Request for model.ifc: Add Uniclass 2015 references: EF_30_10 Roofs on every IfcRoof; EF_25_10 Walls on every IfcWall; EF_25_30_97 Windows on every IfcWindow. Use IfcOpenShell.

First a look at what the model holds.

```python
import ifcopenshell

model = ifcopenshell.open("model.ifc")
print(model.schema)
print("classifications:", [c.Name for c in model.by_type("IfcClassification")])
for ifc_class in ("IfcDoor", "IfcRoof", "IfcStair", "IfcWall", "IfcWindow"):
    print(ifc_class, len(model.by_type(ifc_class)))
```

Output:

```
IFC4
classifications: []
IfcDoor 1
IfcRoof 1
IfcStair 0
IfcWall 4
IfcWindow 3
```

```python
import ifcopenshell
import ifcopenshell.api.classification

model = ifcopenshell.open("model.ifc")

system = ifcopenshell.api.classification.add_classification(model, classification="Uniclass 2015")

codes = {
    "IfcRoof": ("EF_30_10", "Roofs"),
    "IfcWall": ("EF_25_10", "Walls"),
    "IfcWindow": ("EF_25_30_97", "Windows"),
}
for ifc_class, (code, name) in codes.items():
    products = model.by_type(ifc_class)
    ifcopenshell.api.classification.add_reference(
        model, products=products, classification=system, identification=code, name=name
    )
    print(code, len(products))

model.write("model-out.ifc")
```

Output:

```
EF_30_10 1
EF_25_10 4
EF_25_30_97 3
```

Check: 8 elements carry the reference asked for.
